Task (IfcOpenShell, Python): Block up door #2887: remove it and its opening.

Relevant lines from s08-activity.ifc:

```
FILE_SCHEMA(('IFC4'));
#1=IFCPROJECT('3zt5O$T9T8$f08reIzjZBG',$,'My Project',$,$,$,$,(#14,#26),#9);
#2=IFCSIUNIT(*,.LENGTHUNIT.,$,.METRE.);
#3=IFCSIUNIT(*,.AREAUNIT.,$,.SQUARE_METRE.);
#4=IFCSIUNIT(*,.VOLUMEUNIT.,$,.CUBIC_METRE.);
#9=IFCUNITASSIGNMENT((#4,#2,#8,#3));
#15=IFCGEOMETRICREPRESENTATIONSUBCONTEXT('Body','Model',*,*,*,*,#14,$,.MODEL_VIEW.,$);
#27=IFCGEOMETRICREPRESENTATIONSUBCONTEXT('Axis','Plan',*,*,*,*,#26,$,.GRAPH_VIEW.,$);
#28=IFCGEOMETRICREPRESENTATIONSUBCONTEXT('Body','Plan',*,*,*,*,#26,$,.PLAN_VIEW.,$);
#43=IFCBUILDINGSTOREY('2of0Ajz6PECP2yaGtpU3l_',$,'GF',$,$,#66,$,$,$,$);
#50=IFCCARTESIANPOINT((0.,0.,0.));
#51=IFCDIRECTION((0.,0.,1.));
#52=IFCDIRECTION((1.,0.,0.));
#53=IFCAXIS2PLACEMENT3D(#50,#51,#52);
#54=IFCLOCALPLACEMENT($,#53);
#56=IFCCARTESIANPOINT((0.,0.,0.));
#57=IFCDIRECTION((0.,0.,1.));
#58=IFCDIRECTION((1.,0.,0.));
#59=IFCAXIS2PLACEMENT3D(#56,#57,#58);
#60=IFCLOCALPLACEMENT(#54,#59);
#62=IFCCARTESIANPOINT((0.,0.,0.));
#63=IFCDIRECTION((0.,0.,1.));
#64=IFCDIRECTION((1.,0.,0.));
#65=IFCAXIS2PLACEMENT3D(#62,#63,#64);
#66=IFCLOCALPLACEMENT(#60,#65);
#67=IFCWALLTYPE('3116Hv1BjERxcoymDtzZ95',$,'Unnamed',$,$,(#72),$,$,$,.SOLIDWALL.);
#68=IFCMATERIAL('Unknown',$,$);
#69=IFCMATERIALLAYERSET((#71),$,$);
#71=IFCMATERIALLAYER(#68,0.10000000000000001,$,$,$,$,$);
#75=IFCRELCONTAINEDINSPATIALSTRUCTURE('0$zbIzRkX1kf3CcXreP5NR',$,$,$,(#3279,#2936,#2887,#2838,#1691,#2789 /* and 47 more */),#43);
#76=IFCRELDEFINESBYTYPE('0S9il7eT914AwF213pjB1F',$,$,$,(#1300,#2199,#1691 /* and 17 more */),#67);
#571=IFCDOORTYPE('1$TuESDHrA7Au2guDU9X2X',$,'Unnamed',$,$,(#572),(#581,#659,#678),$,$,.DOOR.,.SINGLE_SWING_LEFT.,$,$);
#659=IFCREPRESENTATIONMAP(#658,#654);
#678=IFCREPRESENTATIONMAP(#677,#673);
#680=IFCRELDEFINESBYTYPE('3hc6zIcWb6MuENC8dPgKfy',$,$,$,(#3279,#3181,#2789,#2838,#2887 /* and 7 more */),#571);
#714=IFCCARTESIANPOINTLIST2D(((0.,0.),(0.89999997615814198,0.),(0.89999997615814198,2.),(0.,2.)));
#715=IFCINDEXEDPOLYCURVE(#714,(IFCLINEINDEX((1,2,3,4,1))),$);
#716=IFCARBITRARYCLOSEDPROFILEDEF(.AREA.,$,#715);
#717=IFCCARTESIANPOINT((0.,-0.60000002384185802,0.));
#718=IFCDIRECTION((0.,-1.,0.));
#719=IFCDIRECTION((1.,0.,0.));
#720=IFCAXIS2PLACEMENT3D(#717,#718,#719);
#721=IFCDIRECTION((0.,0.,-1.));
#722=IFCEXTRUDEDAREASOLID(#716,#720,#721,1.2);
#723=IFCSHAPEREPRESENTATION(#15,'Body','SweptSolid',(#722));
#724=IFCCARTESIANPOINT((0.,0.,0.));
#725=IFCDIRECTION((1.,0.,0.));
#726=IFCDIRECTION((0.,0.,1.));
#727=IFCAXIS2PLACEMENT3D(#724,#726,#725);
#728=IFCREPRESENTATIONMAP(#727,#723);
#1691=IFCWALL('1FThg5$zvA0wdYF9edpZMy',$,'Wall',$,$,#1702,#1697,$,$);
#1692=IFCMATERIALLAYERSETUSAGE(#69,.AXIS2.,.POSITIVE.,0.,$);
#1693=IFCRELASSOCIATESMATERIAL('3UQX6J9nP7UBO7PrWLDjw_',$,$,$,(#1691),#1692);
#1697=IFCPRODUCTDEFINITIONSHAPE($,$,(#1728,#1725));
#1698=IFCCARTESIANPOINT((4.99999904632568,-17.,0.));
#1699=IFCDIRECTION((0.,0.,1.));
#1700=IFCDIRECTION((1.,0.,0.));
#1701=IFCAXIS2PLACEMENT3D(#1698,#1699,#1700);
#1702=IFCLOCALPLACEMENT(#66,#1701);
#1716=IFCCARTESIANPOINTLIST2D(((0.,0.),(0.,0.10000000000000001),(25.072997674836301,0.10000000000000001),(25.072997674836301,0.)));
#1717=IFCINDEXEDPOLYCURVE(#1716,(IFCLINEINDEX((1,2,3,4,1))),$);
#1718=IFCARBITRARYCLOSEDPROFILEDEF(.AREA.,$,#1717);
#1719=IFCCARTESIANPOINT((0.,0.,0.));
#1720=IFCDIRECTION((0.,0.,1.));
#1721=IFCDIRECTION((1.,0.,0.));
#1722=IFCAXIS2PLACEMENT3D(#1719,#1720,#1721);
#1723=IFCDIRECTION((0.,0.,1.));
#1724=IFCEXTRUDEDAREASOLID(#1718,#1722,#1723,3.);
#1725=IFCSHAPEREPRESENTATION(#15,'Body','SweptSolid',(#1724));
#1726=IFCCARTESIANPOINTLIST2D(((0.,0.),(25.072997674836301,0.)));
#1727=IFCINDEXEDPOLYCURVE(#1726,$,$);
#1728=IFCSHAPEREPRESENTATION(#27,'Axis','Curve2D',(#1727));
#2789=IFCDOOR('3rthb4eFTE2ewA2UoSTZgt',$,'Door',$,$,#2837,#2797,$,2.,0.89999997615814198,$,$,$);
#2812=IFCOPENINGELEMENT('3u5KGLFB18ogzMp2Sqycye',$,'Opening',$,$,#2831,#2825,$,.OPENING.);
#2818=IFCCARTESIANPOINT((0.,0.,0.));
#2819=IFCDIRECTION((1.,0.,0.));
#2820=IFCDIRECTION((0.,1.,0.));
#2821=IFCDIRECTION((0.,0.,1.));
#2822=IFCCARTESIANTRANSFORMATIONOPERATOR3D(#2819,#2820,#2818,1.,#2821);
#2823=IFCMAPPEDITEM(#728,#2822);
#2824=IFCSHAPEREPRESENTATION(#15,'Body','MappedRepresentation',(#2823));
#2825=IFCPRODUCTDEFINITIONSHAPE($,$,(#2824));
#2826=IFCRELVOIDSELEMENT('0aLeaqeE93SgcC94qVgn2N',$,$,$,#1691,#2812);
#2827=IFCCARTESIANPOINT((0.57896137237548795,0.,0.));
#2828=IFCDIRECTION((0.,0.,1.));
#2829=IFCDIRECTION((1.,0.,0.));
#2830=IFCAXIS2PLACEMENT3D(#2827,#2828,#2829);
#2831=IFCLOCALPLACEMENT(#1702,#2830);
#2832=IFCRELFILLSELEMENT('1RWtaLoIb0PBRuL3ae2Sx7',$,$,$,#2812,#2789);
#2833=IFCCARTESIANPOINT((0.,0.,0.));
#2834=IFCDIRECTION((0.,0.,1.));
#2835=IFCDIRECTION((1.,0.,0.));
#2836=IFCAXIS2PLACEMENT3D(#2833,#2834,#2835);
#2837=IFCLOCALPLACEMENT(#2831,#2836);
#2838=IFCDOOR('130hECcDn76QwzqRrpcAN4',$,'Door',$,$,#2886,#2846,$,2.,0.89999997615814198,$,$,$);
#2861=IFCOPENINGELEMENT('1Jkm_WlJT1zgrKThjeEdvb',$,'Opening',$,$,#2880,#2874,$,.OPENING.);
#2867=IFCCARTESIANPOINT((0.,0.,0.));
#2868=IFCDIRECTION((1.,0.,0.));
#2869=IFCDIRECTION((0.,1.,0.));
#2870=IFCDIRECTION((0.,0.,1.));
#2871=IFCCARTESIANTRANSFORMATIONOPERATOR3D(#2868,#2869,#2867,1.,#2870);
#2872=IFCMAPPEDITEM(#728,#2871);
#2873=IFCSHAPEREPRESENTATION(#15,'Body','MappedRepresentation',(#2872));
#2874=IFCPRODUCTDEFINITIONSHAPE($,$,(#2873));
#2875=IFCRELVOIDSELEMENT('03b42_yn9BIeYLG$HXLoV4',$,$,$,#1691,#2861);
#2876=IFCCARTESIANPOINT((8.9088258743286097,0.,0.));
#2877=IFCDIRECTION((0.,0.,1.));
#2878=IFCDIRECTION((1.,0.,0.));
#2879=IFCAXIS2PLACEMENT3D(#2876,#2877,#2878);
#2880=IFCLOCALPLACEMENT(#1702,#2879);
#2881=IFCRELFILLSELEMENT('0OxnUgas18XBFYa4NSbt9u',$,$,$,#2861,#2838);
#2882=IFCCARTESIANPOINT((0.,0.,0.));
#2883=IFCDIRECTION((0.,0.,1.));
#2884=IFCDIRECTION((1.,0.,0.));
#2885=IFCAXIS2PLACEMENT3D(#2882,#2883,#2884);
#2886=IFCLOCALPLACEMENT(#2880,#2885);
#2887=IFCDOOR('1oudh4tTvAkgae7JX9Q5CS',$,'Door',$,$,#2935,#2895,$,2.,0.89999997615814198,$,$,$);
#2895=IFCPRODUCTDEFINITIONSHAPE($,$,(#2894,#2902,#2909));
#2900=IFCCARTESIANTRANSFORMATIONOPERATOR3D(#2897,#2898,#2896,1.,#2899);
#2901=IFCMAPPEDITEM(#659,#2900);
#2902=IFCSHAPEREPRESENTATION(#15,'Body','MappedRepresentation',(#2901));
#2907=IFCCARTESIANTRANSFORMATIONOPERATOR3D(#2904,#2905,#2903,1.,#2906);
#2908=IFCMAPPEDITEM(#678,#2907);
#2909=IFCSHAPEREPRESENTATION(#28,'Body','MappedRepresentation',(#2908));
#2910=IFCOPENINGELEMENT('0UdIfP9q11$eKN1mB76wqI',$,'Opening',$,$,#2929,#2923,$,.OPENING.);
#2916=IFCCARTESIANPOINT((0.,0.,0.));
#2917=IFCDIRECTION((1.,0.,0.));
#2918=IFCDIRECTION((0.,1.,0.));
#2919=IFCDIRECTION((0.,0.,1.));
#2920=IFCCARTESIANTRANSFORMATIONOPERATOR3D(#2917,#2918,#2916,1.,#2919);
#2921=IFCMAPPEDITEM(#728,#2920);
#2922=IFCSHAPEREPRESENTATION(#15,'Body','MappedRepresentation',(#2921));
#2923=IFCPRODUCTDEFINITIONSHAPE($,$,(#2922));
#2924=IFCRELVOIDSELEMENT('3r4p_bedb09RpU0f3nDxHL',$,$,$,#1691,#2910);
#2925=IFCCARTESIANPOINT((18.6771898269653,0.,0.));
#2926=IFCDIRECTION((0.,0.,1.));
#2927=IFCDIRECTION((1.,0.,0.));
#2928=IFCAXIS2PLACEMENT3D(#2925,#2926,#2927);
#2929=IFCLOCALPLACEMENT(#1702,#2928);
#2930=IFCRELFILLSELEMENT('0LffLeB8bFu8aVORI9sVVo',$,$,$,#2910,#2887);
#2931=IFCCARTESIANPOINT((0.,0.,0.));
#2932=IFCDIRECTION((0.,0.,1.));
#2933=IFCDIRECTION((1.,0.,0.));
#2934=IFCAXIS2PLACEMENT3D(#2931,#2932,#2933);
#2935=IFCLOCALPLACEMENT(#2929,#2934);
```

```python
import ifcopenshell
import ifcopenshell.api.feature
import ifcopenshell.api.root
import ifcopenshell.geom
import ifcopenshell.util.shape

model = ifcopenshell.open("s08-activity.ifc")
settings = ifcopenshell.geom.settings()


def volume(element):
    """Net volume in cubic metres, openings subtracted."""
    shape = ifcopenshell.geom.create_shape(settings, element)
    return ifcopenshell.util.shape.get_volume(shape.geometry)


door = model.by_guid("1oudh4tTvAkgae7JX9Q5CS")
opening = door.FillsVoids[0].RelatingOpeningElement
wall = opening.VoidsElements[0].RelatingBuildingElement
before = volume(wall)

ifcopenshell.api.root.remove_product(model, product=door)
ifcopenshell.api.feature.remove_feature(model, feature=opening)

after = volume(wall)

print(f"wall volume {before:.3f} -> {after:.3f} m3")

model.write("s08-activity_rev.ifc")
```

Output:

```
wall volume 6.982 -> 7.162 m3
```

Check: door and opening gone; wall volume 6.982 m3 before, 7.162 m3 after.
